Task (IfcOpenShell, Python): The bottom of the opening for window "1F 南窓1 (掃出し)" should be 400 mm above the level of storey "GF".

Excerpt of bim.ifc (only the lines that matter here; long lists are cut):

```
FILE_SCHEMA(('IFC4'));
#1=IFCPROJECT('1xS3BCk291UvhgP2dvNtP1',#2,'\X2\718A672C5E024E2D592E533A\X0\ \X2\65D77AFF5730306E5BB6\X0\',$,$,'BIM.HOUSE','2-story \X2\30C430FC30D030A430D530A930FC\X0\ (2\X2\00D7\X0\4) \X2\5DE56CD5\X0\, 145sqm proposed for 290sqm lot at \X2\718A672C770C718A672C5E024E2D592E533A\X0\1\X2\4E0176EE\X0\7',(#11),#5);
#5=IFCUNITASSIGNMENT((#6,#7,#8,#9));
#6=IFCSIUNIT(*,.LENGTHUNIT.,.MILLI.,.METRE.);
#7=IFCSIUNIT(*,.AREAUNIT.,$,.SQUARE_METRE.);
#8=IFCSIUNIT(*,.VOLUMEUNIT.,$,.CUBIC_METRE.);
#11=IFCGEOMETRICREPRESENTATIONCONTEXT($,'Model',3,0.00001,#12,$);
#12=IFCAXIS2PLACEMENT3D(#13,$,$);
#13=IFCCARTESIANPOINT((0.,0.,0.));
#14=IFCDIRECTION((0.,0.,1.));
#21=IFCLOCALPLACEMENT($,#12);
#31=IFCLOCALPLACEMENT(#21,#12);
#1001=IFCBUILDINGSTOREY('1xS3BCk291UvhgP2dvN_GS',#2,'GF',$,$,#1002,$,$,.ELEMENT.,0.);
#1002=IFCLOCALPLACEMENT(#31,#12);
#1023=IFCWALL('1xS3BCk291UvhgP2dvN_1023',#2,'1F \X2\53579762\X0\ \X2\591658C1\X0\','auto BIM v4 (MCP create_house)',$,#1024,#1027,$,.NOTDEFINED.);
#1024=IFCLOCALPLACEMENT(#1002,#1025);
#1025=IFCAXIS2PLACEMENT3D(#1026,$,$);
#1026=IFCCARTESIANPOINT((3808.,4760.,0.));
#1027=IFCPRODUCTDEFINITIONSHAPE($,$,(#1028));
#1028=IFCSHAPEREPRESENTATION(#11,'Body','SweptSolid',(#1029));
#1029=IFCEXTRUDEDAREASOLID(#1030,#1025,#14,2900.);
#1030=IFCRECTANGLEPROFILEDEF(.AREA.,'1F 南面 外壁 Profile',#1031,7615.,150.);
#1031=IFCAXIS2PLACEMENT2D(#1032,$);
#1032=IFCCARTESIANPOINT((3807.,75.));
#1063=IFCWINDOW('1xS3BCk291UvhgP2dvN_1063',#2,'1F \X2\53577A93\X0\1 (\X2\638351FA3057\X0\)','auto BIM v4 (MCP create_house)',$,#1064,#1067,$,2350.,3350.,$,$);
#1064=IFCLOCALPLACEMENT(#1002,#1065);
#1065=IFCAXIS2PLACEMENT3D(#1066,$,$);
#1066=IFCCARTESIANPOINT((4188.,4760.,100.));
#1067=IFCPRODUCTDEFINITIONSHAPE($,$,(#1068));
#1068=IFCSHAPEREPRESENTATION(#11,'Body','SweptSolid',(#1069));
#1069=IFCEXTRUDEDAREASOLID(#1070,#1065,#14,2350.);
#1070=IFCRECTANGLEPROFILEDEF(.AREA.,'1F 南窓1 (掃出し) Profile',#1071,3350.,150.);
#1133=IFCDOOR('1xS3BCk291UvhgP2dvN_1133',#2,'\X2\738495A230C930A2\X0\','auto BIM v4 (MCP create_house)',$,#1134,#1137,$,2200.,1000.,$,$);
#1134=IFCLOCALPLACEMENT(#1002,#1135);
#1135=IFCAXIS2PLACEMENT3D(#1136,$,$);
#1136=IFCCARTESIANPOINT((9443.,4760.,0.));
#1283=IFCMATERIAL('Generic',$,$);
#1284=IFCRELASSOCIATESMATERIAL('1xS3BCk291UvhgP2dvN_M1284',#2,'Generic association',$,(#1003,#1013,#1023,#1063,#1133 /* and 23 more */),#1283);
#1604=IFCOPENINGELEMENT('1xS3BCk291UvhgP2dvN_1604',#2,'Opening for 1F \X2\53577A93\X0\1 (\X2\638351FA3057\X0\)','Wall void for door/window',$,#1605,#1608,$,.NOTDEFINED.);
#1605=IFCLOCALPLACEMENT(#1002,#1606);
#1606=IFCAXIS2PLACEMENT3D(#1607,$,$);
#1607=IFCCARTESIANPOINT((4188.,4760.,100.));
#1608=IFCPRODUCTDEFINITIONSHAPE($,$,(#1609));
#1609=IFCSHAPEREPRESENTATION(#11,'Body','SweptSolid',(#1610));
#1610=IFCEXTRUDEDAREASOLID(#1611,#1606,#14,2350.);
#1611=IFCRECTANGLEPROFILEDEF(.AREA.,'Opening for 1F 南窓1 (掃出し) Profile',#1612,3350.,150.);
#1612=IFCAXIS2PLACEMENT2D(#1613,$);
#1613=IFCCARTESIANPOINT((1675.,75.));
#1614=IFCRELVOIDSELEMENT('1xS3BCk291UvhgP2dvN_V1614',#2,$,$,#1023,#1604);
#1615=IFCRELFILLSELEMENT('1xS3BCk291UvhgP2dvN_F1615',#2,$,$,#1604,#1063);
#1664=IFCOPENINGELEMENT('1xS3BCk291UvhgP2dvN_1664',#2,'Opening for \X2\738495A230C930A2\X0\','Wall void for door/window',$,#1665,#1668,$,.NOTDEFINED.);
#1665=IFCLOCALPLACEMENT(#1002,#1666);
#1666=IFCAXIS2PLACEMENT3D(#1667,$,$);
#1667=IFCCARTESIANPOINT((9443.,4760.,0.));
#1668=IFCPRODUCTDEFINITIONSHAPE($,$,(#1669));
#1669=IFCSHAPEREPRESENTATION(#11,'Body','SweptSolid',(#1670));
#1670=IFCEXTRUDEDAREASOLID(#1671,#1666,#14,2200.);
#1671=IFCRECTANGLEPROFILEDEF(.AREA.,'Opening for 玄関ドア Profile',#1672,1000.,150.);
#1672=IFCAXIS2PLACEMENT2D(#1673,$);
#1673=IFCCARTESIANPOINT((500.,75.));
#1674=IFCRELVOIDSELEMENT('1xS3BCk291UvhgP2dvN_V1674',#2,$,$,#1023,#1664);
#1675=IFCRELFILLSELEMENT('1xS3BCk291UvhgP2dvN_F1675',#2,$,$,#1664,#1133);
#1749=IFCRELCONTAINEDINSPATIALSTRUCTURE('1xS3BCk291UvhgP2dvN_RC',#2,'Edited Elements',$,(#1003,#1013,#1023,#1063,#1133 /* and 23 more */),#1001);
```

```python
import numpy as np
import ifcopenshell
import ifcopenshell.api.geometry
import ifcopenshell.geom
import ifcopenshell.util.element
import ifcopenshell.util.placement
import ifcopenshell.util.shape
import ifcopenshell.util.unit

model = ifcopenshell.open("bim.ifc")
unit_scale = ifcopenshell.util.unit.calculate_unit_scale(model)

window = model.by_guid("1xS3BCk291UvhgP2dvN_1063")
opening = window.FillsVoids[0].RelatingOpeningElement
storey = ifcopenshell.util.element.get_container(window, ifc_class="IfcBuildingStorey")
level = ifcopenshell.util.placement.get_local_placement(storey.ObjectPlacement)[2, 3]

# The opening's origin need not be at the sill, so measure its lowest point.
shape = ifcopenshell.geom.create_shape(ifcopenshell.geom.settings(), opening)
bottom = ifcopenshell.util.shape.get_shape_bottom_elevation(shape, shape.geometry) / unit_scale
dz = level + 0.4 / unit_scale - bottom

shift = np.array([0.0, 0.0, dz])
# The window is not placed relative to its opening, so move both.
for product in (opening, window):
    matrix = ifcopenshell.util.placement.get_local_placement(product.ObjectPlacement)
    matrix[:3, 3] += shift
    ifcopenshell.api.geometry.edit_object_placement(model, product=product, matrix=matrix, is_si=False)

print(f"moved by {dz * unit_scale:+.3f} m")

model.write("bim_edited.ifc")
```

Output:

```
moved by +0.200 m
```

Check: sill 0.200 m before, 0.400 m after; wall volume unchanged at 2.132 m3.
